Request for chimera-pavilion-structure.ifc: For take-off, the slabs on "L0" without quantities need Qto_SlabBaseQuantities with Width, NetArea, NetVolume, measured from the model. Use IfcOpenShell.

First a look at what the model holds.

```python
import ifcopenshell
import ifcopenshell.util.element
import ifcopenshell.util.unit

model = ifcopenshell.open("chimera-pavilion-structure.ifc")
print(model.schema)
for unit_type in ("LENGTHUNIT", "AREAUNIT", "VOLUMEUNIT"):
    print(unit_type, ifcopenshell.util.unit.calculate_unit_scale(model, unit_type))
storey = next(s for s in model.by_type("IfcBuildingStorey") if s.Name == "L0")
slabs = [e for e in ifcopenshell.util.element.get_decomposition(storey) if e.is_a("IfcSlab")]
for e in sorted(slabs, key=lambda e: e.id()):
    print(e.id(), e.is_a(), e.Name, list(ifcopenshell.util.element.get_psets(e, qtos_only=True)), sep=" | ")
```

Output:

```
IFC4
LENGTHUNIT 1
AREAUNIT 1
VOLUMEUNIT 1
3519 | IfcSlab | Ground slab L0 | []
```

```python
import ifcopenshell
import ifcopenshell.api.pset
import ifcopenshell.geom
import ifcopenshell.util.element
import ifcopenshell.util.shape
import ifcopenshell.util.unit

model = ifcopenshell.open("chimera-pavilion-structure.ifc")
unit_scale = ifcopenshell.util.unit.calculate_unit_scale(model)
area_scale = ifcopenshell.util.unit.calculate_unit_scale(model, "AREAUNIT")
volume_scale = ifcopenshell.util.unit.calculate_unit_scale(model, "VOLUMEUNIT")
settings = ifcopenshell.geom.settings()

storey = next(s for s in model.by_type("IfcBuildingStorey") if s.Name == "L0")
slabs = [e for e in ifcopenshell.util.element.get_decomposition(storey) if e.is_a("IfcSlab")]

for e in sorted(slabs, key=lambda e: e.id()):
    if ifcopenshell.util.element.get_psets(e, qtos_only=True, should_inherit=False):
        continue
    # Geometry comes back in metres, in the element's own axes.
    shape = ifcopenshell.geom.create_shape(settings, e)
    values = {
        "Width": ifcopenshell.util.shape.get_z(shape.geometry) / unit_scale,
        "NetArea": ifcopenshell.util.shape.get_footprint_area(shape.geometry) / area_scale,
        "NetVolume": ifcopenshell.util.shape.get_volume(shape.geometry) / volume_scale,
    }
    qto = ifcopenshell.api.pset.add_qto(model, product=e, name="Qto_SlabBaseQuantities")
    ifcopenshell.api.pset.edit_qto(model, qto=qto, properties=values)
    print(e.id(), {k: round(v, 3) for k, v in values.items()})

model.write("chimera-pavilion-structure_edited.ifc")
```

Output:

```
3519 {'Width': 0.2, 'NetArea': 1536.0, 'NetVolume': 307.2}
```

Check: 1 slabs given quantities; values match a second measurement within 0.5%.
